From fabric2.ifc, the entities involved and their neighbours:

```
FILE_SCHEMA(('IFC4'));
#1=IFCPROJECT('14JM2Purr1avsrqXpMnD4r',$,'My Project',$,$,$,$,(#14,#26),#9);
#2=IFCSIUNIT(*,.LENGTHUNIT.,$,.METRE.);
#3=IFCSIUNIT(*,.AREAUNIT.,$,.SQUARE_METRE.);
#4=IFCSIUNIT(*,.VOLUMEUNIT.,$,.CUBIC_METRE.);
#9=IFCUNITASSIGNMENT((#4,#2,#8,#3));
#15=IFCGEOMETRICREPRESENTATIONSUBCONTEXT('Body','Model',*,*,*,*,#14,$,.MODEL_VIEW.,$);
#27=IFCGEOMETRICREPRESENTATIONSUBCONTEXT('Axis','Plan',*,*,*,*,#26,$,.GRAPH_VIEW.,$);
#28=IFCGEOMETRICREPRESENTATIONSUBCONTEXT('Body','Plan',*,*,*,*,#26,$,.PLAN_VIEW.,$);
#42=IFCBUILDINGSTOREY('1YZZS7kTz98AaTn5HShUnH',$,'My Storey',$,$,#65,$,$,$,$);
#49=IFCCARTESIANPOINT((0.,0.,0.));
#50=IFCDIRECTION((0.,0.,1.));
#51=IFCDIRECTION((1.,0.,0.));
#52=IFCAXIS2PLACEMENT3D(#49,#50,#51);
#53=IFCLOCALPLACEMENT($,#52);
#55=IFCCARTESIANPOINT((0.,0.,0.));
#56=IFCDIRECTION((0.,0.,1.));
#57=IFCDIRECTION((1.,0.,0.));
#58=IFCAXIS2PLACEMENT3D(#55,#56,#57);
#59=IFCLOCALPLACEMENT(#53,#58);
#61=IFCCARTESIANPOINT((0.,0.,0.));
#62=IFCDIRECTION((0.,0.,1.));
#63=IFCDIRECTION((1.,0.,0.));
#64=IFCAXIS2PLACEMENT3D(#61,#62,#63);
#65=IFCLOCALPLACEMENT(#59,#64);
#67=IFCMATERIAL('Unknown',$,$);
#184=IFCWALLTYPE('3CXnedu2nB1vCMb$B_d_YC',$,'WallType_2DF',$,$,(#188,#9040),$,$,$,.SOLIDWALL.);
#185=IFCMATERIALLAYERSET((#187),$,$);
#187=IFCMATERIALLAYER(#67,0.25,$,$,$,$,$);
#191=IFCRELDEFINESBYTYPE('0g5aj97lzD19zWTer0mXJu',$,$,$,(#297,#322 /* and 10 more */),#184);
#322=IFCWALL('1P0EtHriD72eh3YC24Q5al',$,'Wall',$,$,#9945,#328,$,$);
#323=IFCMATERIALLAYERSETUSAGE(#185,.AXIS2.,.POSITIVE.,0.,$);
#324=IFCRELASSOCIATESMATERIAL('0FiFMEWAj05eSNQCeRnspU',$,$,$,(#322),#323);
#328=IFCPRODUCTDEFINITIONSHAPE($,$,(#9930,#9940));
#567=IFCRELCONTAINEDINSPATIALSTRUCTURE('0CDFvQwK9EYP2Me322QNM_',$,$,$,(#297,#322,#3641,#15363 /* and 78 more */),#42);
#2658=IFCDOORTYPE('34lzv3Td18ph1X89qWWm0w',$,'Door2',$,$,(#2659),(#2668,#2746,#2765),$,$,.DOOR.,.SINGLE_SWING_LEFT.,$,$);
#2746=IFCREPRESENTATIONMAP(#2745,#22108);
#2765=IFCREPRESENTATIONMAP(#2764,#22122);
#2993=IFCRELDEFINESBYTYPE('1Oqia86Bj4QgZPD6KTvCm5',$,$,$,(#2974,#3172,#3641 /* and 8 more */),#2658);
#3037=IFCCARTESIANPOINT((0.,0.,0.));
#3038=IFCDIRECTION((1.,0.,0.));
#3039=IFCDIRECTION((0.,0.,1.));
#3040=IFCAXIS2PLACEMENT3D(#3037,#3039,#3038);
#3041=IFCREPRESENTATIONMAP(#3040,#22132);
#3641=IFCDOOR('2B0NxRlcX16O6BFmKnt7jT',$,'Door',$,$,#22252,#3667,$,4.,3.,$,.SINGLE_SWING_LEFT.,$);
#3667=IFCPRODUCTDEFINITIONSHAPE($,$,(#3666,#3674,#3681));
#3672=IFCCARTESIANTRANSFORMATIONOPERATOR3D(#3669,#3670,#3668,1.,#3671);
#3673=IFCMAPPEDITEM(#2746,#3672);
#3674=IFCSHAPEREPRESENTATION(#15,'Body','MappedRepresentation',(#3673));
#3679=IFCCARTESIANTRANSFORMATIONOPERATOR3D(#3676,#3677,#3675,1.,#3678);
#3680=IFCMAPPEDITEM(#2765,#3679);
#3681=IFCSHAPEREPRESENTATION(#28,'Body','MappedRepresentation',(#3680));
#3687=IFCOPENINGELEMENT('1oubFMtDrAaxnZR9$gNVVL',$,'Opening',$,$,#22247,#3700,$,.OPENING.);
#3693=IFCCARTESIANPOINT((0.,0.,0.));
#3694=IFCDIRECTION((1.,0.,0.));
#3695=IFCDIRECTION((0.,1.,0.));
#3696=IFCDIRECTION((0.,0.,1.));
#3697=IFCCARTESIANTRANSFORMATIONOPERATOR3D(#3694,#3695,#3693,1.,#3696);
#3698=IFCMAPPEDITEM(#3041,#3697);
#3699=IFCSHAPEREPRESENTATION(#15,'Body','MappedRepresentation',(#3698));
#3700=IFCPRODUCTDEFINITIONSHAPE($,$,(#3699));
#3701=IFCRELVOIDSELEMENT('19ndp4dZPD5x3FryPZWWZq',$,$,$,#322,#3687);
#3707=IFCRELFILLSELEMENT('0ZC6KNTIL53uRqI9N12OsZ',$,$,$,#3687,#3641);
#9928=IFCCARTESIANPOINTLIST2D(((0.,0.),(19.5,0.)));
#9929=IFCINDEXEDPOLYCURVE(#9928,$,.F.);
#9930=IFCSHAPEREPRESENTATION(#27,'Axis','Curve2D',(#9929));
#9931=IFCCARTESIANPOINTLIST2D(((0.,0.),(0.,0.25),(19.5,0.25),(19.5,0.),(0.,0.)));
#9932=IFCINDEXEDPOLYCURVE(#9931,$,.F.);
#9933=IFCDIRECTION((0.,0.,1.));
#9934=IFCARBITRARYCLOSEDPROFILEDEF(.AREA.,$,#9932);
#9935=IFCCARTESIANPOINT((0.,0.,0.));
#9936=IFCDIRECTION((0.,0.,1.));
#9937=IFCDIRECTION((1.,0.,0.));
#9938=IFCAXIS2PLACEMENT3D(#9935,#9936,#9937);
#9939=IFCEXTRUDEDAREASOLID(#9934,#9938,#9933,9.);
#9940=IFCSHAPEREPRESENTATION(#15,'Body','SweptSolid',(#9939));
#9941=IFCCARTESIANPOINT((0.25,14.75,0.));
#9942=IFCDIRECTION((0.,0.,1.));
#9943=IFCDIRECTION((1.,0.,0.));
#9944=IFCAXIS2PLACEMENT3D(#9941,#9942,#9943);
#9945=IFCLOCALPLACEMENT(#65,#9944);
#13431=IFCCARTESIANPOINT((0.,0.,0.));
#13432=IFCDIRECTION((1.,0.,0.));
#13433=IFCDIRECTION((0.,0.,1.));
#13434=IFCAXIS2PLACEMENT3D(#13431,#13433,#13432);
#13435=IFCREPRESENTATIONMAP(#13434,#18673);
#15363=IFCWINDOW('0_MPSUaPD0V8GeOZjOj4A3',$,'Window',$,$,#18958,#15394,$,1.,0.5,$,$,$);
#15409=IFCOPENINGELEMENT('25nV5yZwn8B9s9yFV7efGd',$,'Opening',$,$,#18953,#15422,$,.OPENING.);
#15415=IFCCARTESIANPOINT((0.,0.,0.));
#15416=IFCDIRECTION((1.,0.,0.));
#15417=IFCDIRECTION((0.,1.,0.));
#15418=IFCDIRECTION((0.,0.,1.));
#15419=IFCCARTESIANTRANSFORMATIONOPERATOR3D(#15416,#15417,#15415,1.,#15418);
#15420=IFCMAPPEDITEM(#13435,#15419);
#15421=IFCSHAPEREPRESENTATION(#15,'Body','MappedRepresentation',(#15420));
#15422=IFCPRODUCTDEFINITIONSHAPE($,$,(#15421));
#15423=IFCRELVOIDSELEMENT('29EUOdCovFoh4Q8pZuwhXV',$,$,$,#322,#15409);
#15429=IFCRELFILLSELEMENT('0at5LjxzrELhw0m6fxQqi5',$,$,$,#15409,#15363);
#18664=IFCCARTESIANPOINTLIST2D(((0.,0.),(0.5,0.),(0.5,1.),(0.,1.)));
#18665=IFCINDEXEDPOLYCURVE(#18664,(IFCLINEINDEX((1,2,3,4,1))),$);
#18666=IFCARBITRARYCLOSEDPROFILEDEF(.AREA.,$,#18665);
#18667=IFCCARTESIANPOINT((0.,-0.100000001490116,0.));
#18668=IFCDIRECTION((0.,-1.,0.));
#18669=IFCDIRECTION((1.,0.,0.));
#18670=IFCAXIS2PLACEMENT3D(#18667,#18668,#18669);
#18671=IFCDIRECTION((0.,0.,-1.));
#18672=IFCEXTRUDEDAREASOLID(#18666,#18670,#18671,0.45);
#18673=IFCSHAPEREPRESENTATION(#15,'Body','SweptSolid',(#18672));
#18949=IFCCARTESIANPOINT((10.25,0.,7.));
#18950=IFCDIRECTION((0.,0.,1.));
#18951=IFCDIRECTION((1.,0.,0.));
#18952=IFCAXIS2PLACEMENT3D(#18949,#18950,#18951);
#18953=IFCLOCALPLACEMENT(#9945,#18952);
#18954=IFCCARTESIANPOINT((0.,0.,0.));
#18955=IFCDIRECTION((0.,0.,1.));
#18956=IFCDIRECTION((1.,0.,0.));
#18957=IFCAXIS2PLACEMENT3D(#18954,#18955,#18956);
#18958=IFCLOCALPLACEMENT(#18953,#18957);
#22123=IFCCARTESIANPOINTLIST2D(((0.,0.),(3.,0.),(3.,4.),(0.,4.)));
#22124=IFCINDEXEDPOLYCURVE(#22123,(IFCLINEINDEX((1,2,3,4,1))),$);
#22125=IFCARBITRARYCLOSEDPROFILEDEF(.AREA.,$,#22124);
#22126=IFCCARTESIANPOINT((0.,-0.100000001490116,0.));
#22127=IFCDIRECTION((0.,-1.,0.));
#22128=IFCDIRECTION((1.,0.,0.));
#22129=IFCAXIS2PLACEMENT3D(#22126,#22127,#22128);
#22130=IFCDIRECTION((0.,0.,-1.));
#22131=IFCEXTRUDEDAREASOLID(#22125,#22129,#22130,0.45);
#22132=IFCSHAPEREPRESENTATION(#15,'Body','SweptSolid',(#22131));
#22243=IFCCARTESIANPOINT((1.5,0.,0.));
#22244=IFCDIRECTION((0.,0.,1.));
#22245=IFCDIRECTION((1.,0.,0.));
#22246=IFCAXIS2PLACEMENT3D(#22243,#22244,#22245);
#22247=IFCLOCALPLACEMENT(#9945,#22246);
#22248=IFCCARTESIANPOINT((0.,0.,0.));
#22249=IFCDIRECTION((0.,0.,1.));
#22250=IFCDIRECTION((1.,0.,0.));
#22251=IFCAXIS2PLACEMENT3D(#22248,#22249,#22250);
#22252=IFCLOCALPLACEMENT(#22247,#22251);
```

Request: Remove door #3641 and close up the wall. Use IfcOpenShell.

```python
import ifcopenshell
import ifcopenshell.api.feature
import ifcopenshell.api.root
import ifcopenshell.geom
import ifcopenshell.util.shape

model = ifcopenshell.open("fabric2.ifc")
settings = ifcopenshell.geom.settings()


def volume(element):
    """Net volume in cubic metres, openings subtracted."""
    shape = ifcopenshell.geom.create_shape(settings, element)
    return ifcopenshell.util.shape.get_volume(shape.geometry)


door = model.by_guid("2B0NxRlcX16O6BFmKnt7jT")
opening = door.FillsVoids[0].RelatingOpeningElement
wall = opening.VoidsElements[0].RelatingBuildingElement
before = volume(wall)

ifcopenshell.api.root.remove_product(model, product=door)
ifcopenshell.api.feature.remove_feature(model, feature=opening)

after = volume(wall)

print(f"wall volume {before:.3f} -> {after:.3f} m3")

model.write("fabric2_edited.ifc")
```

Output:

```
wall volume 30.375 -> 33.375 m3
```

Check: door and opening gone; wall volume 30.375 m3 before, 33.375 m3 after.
